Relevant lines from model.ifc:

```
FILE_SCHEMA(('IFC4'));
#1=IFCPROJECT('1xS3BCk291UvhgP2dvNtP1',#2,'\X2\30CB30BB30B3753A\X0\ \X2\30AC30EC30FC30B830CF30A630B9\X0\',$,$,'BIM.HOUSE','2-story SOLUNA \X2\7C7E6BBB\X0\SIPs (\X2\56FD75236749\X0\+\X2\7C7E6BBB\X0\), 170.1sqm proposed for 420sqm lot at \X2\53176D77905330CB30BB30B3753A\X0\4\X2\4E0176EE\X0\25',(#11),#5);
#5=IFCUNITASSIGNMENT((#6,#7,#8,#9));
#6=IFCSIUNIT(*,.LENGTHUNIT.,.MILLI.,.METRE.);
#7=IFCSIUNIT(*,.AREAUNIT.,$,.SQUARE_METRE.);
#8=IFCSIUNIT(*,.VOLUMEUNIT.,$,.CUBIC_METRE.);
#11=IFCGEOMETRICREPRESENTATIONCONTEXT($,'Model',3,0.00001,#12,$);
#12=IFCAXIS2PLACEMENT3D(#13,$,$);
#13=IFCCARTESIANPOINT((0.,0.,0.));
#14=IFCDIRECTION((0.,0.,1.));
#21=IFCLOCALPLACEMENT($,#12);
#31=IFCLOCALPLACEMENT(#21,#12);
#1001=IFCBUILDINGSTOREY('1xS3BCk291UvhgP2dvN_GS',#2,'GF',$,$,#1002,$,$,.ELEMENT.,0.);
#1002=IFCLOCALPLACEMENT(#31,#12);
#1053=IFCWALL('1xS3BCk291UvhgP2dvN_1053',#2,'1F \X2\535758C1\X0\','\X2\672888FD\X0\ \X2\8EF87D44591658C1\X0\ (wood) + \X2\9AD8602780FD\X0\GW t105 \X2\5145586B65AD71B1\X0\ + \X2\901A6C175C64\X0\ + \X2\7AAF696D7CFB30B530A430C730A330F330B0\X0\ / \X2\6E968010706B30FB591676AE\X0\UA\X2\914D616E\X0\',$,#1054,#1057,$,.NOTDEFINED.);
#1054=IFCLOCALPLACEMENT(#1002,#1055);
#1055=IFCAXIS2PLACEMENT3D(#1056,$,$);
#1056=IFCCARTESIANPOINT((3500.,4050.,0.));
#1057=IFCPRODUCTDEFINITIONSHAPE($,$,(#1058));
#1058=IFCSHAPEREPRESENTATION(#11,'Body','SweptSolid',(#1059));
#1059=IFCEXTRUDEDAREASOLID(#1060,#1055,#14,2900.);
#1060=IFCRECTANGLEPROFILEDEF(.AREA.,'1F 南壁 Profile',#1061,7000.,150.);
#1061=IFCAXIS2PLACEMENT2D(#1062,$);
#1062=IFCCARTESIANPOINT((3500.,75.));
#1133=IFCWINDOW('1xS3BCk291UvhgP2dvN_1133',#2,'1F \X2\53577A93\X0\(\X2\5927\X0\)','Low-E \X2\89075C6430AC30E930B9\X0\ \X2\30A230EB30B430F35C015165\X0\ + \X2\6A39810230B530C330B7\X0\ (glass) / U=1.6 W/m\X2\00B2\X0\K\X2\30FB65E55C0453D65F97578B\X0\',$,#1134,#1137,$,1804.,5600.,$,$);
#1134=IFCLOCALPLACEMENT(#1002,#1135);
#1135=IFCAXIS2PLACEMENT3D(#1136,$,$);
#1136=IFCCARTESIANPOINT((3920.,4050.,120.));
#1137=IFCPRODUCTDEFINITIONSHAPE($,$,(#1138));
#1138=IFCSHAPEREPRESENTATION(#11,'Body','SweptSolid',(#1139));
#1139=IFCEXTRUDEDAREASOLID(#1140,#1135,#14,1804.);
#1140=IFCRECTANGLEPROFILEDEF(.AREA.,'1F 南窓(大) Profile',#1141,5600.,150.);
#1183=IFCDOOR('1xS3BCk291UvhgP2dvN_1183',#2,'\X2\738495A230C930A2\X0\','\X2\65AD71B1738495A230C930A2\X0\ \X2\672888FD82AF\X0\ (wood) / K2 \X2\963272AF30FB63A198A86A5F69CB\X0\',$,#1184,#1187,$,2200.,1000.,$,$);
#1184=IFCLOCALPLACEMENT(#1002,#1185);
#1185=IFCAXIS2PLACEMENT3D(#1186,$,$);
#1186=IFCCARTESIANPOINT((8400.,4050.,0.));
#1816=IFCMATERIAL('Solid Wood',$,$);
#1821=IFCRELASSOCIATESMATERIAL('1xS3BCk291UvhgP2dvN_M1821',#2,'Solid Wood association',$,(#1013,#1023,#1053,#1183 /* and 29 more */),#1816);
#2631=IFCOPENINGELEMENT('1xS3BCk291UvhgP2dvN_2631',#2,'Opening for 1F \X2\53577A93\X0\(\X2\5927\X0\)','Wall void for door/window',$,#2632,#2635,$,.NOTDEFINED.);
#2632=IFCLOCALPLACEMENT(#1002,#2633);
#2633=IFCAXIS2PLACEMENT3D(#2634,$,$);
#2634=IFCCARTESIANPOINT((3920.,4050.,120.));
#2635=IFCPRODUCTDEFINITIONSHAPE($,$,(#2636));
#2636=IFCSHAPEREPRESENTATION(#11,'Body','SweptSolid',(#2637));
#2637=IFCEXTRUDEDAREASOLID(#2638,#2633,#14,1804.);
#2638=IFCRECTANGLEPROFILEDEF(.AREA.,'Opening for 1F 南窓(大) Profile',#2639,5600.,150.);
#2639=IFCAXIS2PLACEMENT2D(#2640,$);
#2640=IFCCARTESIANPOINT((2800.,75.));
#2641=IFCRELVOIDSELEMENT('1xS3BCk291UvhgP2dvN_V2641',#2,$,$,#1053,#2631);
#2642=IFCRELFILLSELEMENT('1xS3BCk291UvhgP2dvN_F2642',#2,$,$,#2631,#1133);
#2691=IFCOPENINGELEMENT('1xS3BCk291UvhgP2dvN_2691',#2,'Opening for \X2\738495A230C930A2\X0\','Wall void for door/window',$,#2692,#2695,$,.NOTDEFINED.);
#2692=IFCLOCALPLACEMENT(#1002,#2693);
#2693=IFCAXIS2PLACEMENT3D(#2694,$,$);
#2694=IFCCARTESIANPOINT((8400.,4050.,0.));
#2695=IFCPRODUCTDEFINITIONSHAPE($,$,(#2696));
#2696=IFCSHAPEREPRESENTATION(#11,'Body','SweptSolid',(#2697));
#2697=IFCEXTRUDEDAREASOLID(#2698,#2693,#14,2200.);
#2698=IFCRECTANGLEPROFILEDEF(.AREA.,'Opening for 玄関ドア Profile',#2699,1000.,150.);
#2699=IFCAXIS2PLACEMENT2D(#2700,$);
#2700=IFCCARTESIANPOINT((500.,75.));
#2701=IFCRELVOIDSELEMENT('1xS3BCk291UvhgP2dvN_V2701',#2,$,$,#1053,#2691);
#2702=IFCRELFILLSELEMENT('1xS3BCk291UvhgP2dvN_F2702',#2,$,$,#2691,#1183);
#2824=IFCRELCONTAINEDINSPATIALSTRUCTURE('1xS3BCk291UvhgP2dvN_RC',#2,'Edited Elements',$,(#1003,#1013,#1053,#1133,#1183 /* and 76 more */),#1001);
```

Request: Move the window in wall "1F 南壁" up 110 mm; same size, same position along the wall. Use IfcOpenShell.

```python
import numpy as np
import ifcopenshell
import ifcopenshell.api.geometry
import ifcopenshell.util.placement
import ifcopenshell.util.unit

model = ifcopenshell.open("model.ifc")
unit_scale = ifcopenshell.util.unit.calculate_unit_scale(model)

window = model.by_guid("1xS3BCk291UvhgP2dvN_1133")
opening = window.FillsVoids[0].RelatingOpeningElement
dz = 0.11 / unit_scale

shift = np.array([0.0, 0.0, dz])
# The window is not placed relative to its opening, so move both.
for product in (opening, window):
    matrix = ifcopenshell.util.placement.get_local_placement(product.ObjectPlacement)
    matrix[:3, 3] += shift
    ifcopenshell.api.geometry.edit_object_placement(model, product=product, matrix=matrix, is_si=False)

print(f"moved by {dz * unit_scale:+.3f} m")

model.write("model-out.ifc")
```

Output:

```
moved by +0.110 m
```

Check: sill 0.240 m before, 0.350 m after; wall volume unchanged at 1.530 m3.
